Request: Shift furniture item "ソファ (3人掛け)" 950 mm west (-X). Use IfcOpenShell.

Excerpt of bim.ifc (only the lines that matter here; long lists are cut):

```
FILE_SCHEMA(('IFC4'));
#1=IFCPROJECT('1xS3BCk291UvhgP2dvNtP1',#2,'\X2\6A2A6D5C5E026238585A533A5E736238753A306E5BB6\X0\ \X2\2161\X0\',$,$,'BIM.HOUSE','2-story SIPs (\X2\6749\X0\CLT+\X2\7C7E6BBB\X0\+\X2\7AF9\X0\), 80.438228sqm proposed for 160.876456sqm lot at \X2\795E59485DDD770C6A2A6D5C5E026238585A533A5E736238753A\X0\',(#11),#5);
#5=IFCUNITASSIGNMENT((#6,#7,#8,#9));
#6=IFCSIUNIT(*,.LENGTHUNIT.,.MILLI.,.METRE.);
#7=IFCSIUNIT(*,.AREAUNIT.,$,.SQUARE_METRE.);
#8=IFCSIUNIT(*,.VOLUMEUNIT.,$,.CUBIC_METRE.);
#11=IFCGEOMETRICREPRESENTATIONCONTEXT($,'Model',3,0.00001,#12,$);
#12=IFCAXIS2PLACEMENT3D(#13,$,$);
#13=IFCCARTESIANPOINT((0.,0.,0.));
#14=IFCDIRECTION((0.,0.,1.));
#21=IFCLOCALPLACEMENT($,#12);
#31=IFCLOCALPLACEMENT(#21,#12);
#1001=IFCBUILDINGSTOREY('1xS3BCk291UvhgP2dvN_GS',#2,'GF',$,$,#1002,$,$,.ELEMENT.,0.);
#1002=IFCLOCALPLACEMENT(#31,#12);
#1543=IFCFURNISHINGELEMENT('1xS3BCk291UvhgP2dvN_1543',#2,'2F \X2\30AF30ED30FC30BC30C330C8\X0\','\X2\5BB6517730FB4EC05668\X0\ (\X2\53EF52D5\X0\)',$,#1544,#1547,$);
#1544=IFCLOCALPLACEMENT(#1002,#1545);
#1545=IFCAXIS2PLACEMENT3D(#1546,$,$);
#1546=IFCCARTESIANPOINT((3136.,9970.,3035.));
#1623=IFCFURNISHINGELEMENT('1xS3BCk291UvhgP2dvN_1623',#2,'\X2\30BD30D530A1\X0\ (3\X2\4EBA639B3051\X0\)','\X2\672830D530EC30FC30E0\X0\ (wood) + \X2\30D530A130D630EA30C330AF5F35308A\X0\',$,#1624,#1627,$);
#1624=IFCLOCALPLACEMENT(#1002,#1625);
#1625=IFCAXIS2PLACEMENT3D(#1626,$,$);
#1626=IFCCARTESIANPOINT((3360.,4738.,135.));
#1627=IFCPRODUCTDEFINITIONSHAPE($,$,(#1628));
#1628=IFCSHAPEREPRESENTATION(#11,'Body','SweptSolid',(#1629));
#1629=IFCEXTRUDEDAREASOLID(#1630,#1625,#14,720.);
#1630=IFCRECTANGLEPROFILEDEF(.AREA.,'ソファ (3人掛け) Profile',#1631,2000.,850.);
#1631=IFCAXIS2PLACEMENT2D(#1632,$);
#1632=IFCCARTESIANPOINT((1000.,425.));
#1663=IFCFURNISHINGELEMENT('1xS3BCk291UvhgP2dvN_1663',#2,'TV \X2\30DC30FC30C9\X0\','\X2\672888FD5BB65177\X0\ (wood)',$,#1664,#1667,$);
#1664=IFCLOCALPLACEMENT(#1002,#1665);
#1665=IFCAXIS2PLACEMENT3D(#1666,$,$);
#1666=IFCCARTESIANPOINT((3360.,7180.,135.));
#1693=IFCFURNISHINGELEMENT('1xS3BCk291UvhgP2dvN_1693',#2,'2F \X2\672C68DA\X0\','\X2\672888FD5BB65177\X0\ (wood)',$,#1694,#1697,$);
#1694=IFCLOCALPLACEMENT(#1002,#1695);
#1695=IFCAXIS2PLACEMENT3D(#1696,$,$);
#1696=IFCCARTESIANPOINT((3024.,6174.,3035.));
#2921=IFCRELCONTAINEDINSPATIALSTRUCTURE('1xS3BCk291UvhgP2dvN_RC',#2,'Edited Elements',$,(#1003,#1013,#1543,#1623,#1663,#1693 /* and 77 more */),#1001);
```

```python
import ifcopenshell
import ifcopenshell.api.geometry
import ifcopenshell.util.placement
import ifcopenshell.util.unit

model = ifcopenshell.open("bim.ifc")
unit_scale = ifcopenshell.util.unit.calculate_unit_scale(model)

item = model.by_id(1623)
matrix = ifcopenshell.util.placement.get_local_placement(item.ObjectPlacement)
matrix[0, 3] -= 0.95 / unit_scale
ifcopenshell.api.geometry.edit_object_placement(model, product=item, matrix=matrix, is_si=False)

print(ifcopenshell.util.placement.get_local_placement(item.ObjectPlacement).round(3) + 0.0)

model.write("bim_rev.ifc")
```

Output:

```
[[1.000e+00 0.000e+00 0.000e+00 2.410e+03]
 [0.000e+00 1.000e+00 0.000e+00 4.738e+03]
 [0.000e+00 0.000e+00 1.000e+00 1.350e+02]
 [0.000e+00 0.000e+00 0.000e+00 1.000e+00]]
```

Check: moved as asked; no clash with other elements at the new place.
